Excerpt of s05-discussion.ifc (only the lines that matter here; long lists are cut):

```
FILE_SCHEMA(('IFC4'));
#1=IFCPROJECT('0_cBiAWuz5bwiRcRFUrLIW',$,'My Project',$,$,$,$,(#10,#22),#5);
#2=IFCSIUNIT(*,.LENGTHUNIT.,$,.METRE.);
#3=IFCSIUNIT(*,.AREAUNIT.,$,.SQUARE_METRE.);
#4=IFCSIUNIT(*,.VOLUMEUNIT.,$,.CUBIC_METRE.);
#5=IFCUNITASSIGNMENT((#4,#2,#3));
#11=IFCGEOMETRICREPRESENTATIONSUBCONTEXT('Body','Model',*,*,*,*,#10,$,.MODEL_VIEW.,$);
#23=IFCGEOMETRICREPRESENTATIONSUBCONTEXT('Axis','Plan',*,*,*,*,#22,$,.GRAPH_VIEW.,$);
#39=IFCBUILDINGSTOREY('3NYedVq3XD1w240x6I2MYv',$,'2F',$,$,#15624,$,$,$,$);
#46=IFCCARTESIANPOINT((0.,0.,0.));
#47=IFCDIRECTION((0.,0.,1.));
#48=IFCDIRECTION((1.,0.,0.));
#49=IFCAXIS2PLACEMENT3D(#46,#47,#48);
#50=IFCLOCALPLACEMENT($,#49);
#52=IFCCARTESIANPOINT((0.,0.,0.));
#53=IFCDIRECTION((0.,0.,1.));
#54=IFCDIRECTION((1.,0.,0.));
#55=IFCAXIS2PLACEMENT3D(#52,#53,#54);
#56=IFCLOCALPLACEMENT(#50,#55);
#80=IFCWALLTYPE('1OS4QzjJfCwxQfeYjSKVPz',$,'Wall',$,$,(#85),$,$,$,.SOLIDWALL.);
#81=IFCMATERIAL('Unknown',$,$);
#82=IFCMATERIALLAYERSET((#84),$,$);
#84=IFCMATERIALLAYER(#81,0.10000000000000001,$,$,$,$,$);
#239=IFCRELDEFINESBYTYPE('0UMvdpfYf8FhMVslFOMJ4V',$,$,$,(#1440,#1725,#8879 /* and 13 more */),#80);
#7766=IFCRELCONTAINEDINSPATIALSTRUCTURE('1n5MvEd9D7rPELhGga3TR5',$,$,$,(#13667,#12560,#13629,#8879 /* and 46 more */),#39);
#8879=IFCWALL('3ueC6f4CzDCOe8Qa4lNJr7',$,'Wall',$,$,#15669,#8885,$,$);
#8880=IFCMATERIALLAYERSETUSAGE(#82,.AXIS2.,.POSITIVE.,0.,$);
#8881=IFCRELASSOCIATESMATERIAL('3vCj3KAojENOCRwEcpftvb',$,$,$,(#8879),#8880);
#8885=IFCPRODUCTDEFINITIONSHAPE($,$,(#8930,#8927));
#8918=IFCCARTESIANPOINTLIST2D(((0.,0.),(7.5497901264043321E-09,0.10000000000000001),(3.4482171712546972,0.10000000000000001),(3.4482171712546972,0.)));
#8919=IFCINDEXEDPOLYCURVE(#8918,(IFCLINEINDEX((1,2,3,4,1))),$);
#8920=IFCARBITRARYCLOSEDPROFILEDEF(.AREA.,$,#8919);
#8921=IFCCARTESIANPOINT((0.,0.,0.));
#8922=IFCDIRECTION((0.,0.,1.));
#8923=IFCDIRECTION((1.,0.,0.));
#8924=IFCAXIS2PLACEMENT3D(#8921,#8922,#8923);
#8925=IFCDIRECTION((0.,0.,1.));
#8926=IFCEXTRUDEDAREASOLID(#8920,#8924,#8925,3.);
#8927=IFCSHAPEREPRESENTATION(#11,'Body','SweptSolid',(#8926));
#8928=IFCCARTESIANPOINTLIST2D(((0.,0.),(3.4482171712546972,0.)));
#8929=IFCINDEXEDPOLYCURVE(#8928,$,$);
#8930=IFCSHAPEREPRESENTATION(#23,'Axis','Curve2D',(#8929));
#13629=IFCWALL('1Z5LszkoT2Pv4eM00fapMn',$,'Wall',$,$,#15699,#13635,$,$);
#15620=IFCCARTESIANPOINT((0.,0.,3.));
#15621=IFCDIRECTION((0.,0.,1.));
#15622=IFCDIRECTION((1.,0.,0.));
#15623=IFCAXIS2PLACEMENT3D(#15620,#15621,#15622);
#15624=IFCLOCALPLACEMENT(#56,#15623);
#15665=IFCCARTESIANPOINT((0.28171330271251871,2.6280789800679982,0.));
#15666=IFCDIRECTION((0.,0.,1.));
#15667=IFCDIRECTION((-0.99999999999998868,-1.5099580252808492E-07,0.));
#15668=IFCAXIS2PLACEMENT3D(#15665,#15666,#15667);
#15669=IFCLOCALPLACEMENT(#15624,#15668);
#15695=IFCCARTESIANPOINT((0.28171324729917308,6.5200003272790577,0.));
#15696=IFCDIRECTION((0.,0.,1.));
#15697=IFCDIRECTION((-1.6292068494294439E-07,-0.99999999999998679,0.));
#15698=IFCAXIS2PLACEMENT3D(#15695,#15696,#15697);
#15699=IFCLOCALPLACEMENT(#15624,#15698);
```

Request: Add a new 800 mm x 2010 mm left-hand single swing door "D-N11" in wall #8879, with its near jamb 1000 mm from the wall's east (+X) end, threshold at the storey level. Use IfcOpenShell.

```python
import numpy as np
import ifcopenshell
import ifcopenshell.api.feature
import ifcopenshell.api.geometry
import ifcopenshell.api.root
import ifcopenshell.api.spatial
import ifcopenshell.geom
import ifcopenshell.util.element
import ifcopenshell.util.placement
import ifcopenshell.util.representation
import ifcopenshell.util.shape
import ifcopenshell.util.unit

model = ifcopenshell.open("s05-discussion.ifc")
unit_scale = ifcopenshell.util.unit.calculate_unit_scale(model)
settings = ifcopenshell.geom.settings()


def volume(element):
    """Net volume in cubic metres, openings subtracted."""
    shape = ifcopenshell.geom.create_shape(settings, element)
    return ifcopenshell.util.shape.get_volume(shape.geometry)


wall = model.by_id(8879)
storey = ifcopenshell.util.element.get_container(wall, ifc_class="IfcBuildingStorey")
context = ifcopenshell.util.representation.get_context(model, "Model", "Body", "MODEL_VIEW")
before = volume(wall)

width, height, from_end, sill = 0.8, 2.01, 1, 0.0  # metres

# The wall runs along its own X axis, and the end named is its -X end.
wall_shape = ifcopenshell.geom.create_shape(settings, wall)
x, y, z = ifcopenshell.util.shape.get_vertices(wall_shape.geometry).T
start = x.min() + from_end
face, thickness = float(y.min()), float(y.max() - y.min())
wall_matrix = ifcopenshell.util.placement.get_local_placement(wall.ObjectPlacement)
level = ifcopenshell.util.placement.get_local_placement(storey.ObjectPlacement)[2, 3]


def in_wall(x, y):
    """Placement at x, y metres in the wall's axes, at sill height."""
    matrix = wall_matrix.copy()
    matrix[:, 3] = wall_matrix @ np.array([x / unit_scale, y / unit_scale, 0.0, 1.0])
    matrix[2, 3] = level + sill / unit_scale
    return matrix


# Opening: a box that overshoots both wall faces by 50 mm.
opening = ifcopenshell.api.root.create_entity(model, ifc_class="IfcOpeningElement", predefined_type="OPENING")
box = ifcopenshell.api.geometry.add_wall_representation(
    model, context=context, length=width, height=height, thickness=thickness + 0.1
)
ifcopenshell.api.geometry.assign_representation(model, product=opening, representation=box)
ifcopenshell.api.geometry.edit_object_placement(model, product=opening, matrix=in_wall(start, face - 0.05), is_si=False)
ifcopenshell.api.feature.add_feature(model, feature=opening, element=wall)

door = ifcopenshell.api.root.create_entity(model, ifc_class="IfcDoor", name="D-N11", predefined_type="DOOR")
door.OverallWidth, door.OverallHeight = width / unit_scale, height / unit_scale
door.OperationType = "SINGLE_SWING_LEFT"
body = ifcopenshell.api.geometry.add_door_representation(
    model,
    context=context,
    overall_width=door.OverallWidth,
    overall_height=door.OverallHeight,
    operation_type="SINGLE_SWING_LEFT",
    lining_properties={"LiningDepth": thickness / unit_scale, "ThresholdDepth": thickness / unit_scale},
)
ifcopenshell.api.geometry.assign_representation(model, product=door, representation=body)
ifcopenshell.api.spatial.assign_container(model, products=[door], relating_structure=storey)
ifcopenshell.api.feature.add_filling(model, opening=opening, element=door)

# The lining spans the wall, so the door starts at the wall face.
ifcopenshell.api.geometry.edit_object_placement(model, product=door, matrix=in_wall(start, face), is_si=False)

after = volume(wall)

print(f"wall volume {before:.3f} -> {after:.3f} m3")

model.write("s05-discussion_v2.ifc")
```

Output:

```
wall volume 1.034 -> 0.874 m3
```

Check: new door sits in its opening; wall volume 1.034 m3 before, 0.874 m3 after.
